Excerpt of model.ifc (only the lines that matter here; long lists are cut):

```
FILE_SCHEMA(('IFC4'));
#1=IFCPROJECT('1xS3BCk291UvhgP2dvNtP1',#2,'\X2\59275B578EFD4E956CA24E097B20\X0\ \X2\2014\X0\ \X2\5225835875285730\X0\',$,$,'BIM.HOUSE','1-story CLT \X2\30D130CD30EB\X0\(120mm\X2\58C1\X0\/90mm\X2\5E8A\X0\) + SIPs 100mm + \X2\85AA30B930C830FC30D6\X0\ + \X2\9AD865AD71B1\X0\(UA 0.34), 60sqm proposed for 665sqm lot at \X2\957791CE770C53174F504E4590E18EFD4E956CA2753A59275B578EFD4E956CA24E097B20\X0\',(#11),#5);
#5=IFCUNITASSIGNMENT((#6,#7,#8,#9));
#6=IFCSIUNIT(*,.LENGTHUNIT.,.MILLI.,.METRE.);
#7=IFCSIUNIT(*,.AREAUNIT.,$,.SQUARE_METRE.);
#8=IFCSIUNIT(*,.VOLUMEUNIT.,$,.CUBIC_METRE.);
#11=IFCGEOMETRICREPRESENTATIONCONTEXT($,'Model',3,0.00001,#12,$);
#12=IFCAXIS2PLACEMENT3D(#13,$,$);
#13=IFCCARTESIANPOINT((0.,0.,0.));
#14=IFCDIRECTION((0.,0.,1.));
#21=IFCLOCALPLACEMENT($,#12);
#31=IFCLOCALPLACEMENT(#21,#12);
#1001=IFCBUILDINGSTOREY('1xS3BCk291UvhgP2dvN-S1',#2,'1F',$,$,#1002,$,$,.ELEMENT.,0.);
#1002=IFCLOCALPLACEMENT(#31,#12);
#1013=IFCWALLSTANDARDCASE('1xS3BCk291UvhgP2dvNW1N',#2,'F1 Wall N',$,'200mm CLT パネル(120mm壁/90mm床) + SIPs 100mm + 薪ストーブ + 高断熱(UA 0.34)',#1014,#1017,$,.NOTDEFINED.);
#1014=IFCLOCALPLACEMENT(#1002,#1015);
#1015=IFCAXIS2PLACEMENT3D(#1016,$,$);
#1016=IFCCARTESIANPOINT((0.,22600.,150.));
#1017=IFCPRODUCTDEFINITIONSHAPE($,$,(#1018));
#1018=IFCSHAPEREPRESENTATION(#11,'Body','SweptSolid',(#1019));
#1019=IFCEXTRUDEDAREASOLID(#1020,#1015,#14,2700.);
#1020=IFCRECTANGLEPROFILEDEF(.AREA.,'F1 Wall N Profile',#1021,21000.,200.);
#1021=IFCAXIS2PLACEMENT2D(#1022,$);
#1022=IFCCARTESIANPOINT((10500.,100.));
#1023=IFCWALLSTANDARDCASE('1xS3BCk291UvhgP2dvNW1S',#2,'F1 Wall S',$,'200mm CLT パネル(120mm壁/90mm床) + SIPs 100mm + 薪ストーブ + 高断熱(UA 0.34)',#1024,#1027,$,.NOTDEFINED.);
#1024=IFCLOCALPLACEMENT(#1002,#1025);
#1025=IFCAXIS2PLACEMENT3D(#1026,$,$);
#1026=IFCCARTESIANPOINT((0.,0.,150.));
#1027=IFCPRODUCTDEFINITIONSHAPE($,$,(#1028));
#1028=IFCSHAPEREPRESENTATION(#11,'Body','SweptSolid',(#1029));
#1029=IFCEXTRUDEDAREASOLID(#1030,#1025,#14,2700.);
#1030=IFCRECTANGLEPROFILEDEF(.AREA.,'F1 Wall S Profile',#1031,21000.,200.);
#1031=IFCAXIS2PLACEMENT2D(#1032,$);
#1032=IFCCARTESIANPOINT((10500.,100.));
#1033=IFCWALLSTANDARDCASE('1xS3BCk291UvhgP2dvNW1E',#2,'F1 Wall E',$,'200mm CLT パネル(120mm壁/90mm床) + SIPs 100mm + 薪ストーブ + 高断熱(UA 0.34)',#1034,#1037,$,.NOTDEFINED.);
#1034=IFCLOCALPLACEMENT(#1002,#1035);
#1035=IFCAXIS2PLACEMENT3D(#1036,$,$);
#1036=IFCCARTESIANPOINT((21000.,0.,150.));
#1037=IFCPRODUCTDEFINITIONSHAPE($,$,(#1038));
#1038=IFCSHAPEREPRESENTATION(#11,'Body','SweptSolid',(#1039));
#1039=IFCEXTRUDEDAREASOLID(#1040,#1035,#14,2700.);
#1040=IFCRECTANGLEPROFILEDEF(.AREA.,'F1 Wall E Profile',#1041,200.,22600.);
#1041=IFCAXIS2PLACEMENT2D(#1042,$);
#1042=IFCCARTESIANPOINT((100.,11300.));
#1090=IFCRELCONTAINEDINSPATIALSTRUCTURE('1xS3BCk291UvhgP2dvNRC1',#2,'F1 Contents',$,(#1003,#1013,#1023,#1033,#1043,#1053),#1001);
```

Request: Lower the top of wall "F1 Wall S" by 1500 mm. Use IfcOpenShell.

```python
import ifcopenshell
import ifcopenshell.geom
import ifcopenshell.util.shape
import ifcopenshell.util.unit

model = ifcopenshell.open("model.ifc")
unit_scale = ifcopenshell.util.unit.calculate_unit_scale(model)
settings = ifcopenshell.geom.settings()


def volume(element):
    """Net volume in cubic metres, openings subtracted."""
    shape = ifcopenshell.geom.create_shape(settings, element)
    return ifcopenshell.util.shape.get_volume(shape.geometry)


wall = model.by_id(1023)
before = volume(wall)

body = next(r for r in wall.Representation.Representations if r.RepresentationIdentifier == "Body")
solid = body.Items[0]
old_height = solid.Depth
solid.Depth -= 1.5 / unit_scale
after = volume(wall)

print(f"height {old_height:g} -> {solid.Depth:g}, volume {before:.3f} -> {after:.3f} m3")

model.write("model_v2.ifc")
```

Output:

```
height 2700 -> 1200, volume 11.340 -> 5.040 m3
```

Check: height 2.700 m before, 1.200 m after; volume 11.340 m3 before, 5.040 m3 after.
